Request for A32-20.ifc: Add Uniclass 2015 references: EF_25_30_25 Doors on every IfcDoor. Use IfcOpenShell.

First a look at what the model holds.

```python
import ifcopenshell

model = ifcopenshell.open("A32-20.ifc")
print(model.schema)
print("classifications:", [c.Name for c in model.by_type("IfcClassification")])
for ifc_class in ("IfcDoor", "IfcRoof", "IfcStair", "IfcWall", "IfcWindow"):
    print(ifc_class, len(model.by_type(ifc_class)))
```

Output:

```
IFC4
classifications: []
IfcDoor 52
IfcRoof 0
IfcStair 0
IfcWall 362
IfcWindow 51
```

```python
import ifcopenshell
import ifcopenshell.api.classification

model = ifcopenshell.open("A32-20.ifc")

system = ifcopenshell.api.classification.add_classification(model, classification="Uniclass 2015")

codes = {
    "IfcDoor": ("EF_25_30_25", "Doors"),
}
for ifc_class, (code, name) in codes.items():
    products = model.by_type(ifc_class)
    ifcopenshell.api.classification.add_reference(
        model, products=products, classification=system, identification=code, name=name
    )
    print(code, len(products))

model.write("A32-20_updated.ifc")
```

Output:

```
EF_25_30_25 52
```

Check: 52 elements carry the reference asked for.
